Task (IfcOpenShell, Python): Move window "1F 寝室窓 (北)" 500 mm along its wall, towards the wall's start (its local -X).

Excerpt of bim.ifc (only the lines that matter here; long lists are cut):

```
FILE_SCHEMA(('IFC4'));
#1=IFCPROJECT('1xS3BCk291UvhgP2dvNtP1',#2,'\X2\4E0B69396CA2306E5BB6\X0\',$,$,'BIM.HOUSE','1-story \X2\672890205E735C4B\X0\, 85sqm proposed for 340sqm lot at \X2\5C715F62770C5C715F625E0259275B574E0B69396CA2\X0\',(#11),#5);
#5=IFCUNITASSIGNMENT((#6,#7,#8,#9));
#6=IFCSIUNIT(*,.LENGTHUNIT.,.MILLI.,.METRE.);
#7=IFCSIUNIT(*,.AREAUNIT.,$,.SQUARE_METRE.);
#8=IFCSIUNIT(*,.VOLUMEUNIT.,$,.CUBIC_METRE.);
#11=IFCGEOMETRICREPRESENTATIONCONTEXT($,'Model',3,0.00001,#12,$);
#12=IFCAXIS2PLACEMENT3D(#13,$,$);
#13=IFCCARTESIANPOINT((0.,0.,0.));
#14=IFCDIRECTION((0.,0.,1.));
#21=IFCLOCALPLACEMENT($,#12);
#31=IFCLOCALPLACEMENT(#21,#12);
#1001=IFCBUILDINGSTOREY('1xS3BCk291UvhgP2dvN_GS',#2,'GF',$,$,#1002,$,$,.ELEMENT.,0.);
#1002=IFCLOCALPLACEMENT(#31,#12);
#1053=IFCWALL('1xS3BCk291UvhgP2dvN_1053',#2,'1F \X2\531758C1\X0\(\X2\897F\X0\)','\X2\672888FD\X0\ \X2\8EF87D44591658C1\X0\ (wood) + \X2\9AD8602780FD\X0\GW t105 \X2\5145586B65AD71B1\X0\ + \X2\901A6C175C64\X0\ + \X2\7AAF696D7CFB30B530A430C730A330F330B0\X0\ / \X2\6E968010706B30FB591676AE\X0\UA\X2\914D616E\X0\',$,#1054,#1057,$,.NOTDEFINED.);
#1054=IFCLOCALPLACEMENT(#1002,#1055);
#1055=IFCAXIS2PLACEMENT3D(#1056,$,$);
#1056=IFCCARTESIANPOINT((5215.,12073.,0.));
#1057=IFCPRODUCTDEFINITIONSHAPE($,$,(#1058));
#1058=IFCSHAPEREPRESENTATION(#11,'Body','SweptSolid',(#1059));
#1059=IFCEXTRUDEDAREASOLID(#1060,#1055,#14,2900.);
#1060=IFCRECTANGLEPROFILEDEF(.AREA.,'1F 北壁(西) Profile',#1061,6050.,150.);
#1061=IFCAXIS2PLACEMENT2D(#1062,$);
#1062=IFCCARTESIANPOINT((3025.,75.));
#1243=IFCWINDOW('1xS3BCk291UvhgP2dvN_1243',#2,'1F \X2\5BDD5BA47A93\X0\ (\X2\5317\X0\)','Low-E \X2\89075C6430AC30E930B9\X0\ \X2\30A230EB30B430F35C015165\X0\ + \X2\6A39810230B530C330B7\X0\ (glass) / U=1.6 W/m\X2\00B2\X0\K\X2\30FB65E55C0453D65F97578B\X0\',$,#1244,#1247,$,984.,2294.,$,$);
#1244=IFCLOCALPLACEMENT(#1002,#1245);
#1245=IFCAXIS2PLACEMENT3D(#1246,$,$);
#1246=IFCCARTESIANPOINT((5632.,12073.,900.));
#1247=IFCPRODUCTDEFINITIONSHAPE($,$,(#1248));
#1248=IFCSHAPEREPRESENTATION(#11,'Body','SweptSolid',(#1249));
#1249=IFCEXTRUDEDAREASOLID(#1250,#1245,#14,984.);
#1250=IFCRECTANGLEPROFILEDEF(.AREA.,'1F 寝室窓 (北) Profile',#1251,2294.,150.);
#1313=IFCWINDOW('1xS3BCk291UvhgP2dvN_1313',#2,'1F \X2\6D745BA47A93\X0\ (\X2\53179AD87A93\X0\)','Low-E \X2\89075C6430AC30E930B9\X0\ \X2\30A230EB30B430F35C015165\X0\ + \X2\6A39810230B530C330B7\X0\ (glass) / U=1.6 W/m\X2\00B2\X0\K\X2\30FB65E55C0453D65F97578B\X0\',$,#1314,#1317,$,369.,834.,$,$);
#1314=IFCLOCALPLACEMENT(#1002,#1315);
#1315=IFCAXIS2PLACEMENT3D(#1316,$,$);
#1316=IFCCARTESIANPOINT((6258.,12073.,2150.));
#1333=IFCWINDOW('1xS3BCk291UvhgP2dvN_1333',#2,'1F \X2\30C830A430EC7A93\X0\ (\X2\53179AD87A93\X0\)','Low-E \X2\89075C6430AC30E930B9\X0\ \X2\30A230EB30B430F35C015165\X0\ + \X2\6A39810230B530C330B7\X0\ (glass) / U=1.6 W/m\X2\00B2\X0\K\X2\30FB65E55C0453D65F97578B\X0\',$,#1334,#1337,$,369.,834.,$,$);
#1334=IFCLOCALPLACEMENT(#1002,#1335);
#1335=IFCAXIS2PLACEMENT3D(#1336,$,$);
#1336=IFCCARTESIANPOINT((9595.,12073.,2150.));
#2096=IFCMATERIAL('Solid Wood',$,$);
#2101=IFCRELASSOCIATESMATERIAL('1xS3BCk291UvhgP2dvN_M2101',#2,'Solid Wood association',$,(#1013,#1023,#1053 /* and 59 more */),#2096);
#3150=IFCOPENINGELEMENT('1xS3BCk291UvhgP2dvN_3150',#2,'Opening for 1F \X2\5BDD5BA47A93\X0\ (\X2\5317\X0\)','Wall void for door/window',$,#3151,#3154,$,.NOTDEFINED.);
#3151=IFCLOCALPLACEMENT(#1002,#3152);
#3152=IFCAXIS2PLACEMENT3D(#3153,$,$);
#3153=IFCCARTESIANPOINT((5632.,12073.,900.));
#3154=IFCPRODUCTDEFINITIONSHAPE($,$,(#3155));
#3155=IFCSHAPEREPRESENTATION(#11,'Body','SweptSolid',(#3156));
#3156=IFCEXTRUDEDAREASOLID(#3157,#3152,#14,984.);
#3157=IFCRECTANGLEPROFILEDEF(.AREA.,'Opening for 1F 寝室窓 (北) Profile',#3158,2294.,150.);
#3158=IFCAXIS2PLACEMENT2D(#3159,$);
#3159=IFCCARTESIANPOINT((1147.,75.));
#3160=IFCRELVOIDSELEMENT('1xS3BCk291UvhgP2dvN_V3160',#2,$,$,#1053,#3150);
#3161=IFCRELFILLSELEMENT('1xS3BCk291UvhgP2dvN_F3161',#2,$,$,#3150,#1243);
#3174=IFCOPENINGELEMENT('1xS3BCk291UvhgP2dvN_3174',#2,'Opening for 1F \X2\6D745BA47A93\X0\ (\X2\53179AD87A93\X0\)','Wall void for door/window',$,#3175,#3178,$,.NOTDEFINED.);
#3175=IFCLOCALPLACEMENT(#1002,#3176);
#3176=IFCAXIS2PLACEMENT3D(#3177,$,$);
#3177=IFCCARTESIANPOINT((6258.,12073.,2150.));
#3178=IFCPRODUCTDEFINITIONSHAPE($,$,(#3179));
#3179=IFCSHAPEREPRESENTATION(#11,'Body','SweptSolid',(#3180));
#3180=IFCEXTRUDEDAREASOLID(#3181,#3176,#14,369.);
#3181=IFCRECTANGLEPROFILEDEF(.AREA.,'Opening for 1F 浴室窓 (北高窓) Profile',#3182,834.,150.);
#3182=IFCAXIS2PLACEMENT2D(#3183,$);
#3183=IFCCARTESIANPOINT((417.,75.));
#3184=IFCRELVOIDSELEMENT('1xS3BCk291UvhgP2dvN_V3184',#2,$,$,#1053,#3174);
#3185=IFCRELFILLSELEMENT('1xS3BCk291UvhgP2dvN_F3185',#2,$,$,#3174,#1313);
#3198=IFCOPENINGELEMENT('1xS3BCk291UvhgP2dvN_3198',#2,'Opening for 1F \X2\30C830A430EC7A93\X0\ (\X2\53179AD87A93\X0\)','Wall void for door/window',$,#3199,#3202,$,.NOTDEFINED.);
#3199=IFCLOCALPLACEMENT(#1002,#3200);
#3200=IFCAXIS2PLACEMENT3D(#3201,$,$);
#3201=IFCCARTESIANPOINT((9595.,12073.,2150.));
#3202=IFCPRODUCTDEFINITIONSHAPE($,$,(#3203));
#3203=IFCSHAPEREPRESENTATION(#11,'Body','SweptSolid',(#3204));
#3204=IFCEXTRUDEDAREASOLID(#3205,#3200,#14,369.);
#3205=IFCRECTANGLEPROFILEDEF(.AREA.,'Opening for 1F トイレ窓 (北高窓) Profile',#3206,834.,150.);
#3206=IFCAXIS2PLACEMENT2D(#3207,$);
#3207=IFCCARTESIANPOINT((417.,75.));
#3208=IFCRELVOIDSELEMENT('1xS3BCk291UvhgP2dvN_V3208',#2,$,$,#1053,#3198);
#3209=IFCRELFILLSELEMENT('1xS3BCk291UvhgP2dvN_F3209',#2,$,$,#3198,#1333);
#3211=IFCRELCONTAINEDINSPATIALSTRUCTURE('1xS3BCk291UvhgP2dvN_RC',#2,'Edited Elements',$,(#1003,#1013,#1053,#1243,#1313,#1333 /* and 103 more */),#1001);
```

```python
import ifcopenshell
import ifcopenshell.api.geometry
import ifcopenshell.util.placement

model = ifcopenshell.open("bim.ifc")

window = model.by_guid("1xS3BCk291UvhgP2dvN_1243")
opening = window.FillsVoids[0].RelatingOpeningElement
wall = opening.VoidsElements[0].RelatingBuildingElement

wall_matrix = ifcopenshell.util.placement.get_local_placement(wall.ObjectPlacement)
shift = wall_matrix[:3, 0] * -500.0
before = ifcopenshell.util.placement.get_local_placement(window.ObjectPlacement)[:3, 3].copy()

# The window is not placed relative to its opening, so move both.
for product in (opening, window):
    matrix = ifcopenshell.util.placement.get_local_placement(product.ObjectPlacement)
    matrix[:3, 3] += shift
    ifcopenshell.api.geometry.edit_object_placement(model, product=product, matrix=matrix, is_si=False)

after = ifcopenshell.util.placement.get_local_placement(window.ObjectPlacement)[:3, 3]
print("window moved by", (after - before).round(3) + 0.0)

model.write("bim-out.ifc")
```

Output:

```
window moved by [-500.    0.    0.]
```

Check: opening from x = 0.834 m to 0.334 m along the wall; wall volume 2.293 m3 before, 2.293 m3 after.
